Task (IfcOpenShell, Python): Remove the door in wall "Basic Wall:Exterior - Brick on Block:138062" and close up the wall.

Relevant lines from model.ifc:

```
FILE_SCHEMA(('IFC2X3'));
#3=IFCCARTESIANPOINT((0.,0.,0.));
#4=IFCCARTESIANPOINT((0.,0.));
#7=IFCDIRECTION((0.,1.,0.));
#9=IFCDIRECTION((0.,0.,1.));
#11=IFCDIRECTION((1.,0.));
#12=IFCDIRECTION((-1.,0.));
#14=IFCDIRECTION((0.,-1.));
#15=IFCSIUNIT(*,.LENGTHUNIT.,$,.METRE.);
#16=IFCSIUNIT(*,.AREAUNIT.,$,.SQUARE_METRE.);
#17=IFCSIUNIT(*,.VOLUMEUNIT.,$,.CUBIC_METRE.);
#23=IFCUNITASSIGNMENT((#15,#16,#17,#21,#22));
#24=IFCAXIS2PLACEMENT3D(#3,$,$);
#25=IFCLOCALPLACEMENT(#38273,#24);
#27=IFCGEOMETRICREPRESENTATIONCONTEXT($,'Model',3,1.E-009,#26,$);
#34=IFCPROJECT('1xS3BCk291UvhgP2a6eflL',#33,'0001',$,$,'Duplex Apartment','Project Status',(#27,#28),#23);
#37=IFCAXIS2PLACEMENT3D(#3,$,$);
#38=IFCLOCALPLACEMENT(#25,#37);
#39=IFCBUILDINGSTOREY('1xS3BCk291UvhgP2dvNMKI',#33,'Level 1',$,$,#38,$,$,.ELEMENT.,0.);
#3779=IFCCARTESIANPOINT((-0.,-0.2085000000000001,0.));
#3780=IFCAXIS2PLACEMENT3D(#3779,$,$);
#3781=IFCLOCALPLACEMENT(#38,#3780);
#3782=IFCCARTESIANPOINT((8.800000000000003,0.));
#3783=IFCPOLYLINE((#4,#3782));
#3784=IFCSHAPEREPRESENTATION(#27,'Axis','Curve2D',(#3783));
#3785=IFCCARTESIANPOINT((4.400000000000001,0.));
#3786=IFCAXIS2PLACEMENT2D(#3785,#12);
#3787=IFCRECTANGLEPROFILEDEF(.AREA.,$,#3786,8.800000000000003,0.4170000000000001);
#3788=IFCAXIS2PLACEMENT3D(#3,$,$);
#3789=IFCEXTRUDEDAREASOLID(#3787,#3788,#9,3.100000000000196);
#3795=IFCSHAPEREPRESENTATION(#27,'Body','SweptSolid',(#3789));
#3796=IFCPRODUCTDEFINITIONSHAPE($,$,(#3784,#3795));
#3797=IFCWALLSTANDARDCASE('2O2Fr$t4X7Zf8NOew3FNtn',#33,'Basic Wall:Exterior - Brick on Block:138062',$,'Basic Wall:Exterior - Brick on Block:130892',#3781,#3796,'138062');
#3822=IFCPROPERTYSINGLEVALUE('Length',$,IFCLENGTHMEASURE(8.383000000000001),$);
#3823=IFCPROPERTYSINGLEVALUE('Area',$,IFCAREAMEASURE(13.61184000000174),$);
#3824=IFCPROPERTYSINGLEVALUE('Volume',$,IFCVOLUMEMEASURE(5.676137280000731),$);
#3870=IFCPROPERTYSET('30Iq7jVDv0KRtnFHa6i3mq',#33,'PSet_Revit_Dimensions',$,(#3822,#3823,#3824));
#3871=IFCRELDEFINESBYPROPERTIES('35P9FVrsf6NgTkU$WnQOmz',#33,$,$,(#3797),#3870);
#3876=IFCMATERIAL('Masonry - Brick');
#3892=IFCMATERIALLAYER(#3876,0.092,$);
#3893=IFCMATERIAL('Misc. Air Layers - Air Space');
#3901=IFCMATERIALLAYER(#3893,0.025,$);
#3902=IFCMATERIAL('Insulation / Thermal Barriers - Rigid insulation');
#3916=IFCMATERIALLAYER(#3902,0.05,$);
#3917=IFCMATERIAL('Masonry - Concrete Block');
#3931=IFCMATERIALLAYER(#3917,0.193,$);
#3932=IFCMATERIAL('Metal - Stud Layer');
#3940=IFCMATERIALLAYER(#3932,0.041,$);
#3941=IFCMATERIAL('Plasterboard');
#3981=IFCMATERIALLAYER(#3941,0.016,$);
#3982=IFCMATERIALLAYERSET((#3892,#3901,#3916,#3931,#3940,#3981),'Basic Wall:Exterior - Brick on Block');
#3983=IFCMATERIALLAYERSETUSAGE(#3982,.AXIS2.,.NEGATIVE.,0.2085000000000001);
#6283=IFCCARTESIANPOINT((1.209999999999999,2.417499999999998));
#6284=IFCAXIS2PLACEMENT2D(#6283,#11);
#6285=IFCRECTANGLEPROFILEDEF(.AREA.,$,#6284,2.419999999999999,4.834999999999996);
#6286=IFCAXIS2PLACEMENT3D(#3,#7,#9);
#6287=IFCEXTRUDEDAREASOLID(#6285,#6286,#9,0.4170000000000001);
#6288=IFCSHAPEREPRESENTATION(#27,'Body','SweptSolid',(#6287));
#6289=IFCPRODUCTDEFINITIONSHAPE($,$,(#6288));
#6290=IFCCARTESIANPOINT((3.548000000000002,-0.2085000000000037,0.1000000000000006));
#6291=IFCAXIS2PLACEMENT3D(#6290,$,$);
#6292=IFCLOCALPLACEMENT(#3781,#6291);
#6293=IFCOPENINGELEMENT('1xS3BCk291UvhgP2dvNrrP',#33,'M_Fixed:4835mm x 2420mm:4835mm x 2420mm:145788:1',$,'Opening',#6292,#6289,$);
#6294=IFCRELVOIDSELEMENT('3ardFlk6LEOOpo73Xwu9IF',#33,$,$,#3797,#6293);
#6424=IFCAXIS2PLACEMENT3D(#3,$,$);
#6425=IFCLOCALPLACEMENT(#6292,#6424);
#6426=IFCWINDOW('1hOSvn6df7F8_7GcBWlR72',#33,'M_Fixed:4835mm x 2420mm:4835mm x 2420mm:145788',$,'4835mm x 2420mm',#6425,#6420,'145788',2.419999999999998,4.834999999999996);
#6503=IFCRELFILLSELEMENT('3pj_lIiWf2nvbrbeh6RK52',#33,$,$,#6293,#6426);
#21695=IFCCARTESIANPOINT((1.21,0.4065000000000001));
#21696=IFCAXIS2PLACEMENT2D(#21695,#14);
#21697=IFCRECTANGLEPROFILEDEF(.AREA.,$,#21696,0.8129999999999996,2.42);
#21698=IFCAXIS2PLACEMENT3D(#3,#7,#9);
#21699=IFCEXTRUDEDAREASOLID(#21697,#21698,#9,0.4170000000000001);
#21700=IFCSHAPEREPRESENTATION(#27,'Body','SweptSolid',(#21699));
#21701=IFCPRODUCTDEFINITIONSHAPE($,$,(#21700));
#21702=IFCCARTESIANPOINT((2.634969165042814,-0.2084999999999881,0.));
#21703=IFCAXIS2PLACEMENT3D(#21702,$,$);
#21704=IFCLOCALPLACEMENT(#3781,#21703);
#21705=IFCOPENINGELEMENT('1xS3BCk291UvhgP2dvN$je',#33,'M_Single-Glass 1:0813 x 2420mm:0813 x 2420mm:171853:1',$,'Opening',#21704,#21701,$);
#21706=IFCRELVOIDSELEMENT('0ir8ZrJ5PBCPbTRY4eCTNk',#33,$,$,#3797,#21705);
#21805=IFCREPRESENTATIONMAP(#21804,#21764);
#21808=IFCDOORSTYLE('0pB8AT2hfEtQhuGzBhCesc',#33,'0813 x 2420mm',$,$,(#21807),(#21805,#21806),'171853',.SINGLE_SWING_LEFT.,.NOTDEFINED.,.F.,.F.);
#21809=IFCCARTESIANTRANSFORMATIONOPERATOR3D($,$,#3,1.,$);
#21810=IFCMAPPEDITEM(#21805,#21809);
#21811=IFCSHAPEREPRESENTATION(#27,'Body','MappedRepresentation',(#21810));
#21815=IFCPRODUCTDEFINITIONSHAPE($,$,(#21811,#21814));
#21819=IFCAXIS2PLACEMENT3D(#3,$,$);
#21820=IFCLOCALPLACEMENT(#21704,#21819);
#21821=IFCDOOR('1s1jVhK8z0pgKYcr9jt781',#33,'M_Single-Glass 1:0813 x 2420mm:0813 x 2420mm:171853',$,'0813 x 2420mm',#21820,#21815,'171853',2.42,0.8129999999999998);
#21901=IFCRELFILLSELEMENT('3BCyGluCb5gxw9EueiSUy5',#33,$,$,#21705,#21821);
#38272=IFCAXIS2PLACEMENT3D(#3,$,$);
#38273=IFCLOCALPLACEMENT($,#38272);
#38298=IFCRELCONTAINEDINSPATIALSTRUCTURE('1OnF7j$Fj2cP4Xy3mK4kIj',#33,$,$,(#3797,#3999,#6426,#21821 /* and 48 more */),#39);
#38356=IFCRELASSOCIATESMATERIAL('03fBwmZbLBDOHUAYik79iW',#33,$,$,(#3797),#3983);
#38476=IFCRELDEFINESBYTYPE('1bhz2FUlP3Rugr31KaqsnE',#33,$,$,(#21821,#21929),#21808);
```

```python
import ifcopenshell
import ifcopenshell.api.feature
import ifcopenshell.api.pset
import ifcopenshell.api.root
import ifcopenshell.geom
import ifcopenshell.util.element
import ifcopenshell.util.shape
import ifcopenshell.util.unit

model = ifcopenshell.open("model.ifc")
area_scale = ifcopenshell.util.unit.calculate_unit_scale(model, "AREAUNIT")
volume_scale = ifcopenshell.util.unit.calculate_unit_scale(model, "VOLUMEUNIT")
settings = ifcopenshell.geom.settings()


def volume(element):
    """Net volume in cubic metres, openings subtracted."""
    shape = ifcopenshell.geom.create_shape(settings, element)
    return ifcopenshell.util.shape.get_volume(shape.geometry)


door = model.by_guid("1s1jVhK8z0pgKYcr9jt781")
opening = door.FillsVoids[0].RelatingOpeningElement
wall = opening.VoidsElements[0].RelatingBuildingElement
before = volume(wall)

ifcopenshell.api.root.remove_product(model, product=door)
ifcopenshell.api.feature.remove_feature(model, feature=opening)

after = volume(wall)
thickness = 0.417  # wall thickness in metres

# Update the wall's stored quantities.
pset = model.by_id(ifcopenshell.util.element.get_pset(wall, "PSet_Revit_Dimensions", should_inherit=False)["id"])
ifcopenshell.api.pset.edit_pset(model, pset=pset, properties={
    "Area": model.create_entity("IfcAreaMeasure", after / thickness / area_scale),
    "Volume": model.create_entity("IfcVolumeMeasure", after / volume_scale),
})

print(f"wall volume {before:.3f} -> {after:.3f} m3")

model.write("model_v2.ifc")
```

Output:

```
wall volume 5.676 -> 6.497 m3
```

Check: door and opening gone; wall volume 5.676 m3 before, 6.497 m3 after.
